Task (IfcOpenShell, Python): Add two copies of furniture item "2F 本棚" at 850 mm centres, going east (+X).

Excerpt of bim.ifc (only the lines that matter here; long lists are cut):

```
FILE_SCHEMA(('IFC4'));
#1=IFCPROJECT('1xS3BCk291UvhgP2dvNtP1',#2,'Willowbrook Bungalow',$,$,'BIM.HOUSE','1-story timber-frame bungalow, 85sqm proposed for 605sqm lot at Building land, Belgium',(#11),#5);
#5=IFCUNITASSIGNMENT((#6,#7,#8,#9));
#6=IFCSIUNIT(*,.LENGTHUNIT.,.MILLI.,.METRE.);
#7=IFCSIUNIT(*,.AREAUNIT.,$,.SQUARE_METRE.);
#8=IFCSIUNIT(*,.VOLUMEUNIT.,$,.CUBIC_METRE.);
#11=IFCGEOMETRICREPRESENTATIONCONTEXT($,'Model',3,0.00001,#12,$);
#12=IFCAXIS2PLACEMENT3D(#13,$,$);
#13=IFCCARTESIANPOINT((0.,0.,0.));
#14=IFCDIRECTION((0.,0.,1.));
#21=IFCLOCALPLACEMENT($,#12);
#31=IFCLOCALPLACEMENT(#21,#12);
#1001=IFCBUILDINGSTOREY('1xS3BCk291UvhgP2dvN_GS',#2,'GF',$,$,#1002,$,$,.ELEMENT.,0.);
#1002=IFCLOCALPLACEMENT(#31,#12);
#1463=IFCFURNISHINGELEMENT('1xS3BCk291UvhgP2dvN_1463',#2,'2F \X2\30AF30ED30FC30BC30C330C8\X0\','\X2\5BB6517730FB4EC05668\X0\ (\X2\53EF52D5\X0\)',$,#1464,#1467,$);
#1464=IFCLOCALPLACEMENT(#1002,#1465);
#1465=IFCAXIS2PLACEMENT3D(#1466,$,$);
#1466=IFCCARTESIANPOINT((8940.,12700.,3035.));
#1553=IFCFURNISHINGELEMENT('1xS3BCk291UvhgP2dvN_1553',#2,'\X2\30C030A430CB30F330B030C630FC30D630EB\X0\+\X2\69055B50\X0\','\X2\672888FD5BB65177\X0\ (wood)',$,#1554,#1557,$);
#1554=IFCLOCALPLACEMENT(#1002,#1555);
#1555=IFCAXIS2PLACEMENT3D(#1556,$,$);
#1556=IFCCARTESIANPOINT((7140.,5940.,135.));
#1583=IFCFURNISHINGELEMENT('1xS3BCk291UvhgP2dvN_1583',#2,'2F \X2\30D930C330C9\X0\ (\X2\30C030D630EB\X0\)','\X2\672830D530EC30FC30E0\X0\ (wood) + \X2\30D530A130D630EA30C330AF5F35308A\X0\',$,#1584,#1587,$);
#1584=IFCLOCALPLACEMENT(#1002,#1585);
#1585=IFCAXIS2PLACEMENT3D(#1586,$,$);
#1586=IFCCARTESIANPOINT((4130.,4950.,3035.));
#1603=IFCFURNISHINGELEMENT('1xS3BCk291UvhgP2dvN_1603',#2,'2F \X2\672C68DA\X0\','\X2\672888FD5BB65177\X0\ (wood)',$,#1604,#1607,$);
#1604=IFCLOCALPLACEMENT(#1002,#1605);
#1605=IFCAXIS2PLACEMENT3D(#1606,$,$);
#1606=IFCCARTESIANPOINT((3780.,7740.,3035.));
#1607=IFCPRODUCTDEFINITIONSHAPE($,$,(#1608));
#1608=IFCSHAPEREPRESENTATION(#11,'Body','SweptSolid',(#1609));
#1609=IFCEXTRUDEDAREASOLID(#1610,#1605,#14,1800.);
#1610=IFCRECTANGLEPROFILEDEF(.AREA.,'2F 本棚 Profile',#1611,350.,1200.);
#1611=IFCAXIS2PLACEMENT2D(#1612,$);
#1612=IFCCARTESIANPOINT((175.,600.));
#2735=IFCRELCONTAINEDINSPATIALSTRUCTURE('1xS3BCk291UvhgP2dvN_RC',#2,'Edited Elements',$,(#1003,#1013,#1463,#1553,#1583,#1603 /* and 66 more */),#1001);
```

```python
import numpy as np
import ifcopenshell
import ifcopenshell.api.geometry
import ifcopenshell.api.root
import ifcopenshell.util.element
import ifcopenshell.util.placement

model = ifcopenshell.open("bim.ifc")


def reuse_history(source, copy):
    """copy_class also copies each property set's owner history, people and application; keep the originals."""
    for rel in copy.IsDefinedBy:
        if rel.is_a("IfcRelDefinesByProperties") and (history := rel.RelatingPropertyDefinition.OwnerHistory):
            rel.RelatingPropertyDefinition.OwnerHistory = source.OwnerHistory
            ifcopenshell.util.element.remove_deep2(model, history)


source = model.by_id(1603)
base = ifcopenshell.util.placement.get_local_placement(source.ObjectPlacement)
step = np.array([1.0, 0.0, 0.0]) * 850.0

for i in range(1, 3):
    copy = ifcopenshell.api.root.copy_class(model, product=source)
    copy.Representation = ifcopenshell.util.element.copy_deep(
        model, source.Representation, exclude=["IfcGeometricRepresentationContext", "IfcRepresentationMap"]
    )
    reuse_history(source, copy)
    matrix = base.copy()
    matrix[:3, 3] += i * step
    print("added at", matrix[:3, 3].round(3) + 0.0)
    ifcopenshell.api.geometry.edit_object_placement(model, product=copy, matrix=matrix, is_si=False)

model.write("bim_updated.ifc")
```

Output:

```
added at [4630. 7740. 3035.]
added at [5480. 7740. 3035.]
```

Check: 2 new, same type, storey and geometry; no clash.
